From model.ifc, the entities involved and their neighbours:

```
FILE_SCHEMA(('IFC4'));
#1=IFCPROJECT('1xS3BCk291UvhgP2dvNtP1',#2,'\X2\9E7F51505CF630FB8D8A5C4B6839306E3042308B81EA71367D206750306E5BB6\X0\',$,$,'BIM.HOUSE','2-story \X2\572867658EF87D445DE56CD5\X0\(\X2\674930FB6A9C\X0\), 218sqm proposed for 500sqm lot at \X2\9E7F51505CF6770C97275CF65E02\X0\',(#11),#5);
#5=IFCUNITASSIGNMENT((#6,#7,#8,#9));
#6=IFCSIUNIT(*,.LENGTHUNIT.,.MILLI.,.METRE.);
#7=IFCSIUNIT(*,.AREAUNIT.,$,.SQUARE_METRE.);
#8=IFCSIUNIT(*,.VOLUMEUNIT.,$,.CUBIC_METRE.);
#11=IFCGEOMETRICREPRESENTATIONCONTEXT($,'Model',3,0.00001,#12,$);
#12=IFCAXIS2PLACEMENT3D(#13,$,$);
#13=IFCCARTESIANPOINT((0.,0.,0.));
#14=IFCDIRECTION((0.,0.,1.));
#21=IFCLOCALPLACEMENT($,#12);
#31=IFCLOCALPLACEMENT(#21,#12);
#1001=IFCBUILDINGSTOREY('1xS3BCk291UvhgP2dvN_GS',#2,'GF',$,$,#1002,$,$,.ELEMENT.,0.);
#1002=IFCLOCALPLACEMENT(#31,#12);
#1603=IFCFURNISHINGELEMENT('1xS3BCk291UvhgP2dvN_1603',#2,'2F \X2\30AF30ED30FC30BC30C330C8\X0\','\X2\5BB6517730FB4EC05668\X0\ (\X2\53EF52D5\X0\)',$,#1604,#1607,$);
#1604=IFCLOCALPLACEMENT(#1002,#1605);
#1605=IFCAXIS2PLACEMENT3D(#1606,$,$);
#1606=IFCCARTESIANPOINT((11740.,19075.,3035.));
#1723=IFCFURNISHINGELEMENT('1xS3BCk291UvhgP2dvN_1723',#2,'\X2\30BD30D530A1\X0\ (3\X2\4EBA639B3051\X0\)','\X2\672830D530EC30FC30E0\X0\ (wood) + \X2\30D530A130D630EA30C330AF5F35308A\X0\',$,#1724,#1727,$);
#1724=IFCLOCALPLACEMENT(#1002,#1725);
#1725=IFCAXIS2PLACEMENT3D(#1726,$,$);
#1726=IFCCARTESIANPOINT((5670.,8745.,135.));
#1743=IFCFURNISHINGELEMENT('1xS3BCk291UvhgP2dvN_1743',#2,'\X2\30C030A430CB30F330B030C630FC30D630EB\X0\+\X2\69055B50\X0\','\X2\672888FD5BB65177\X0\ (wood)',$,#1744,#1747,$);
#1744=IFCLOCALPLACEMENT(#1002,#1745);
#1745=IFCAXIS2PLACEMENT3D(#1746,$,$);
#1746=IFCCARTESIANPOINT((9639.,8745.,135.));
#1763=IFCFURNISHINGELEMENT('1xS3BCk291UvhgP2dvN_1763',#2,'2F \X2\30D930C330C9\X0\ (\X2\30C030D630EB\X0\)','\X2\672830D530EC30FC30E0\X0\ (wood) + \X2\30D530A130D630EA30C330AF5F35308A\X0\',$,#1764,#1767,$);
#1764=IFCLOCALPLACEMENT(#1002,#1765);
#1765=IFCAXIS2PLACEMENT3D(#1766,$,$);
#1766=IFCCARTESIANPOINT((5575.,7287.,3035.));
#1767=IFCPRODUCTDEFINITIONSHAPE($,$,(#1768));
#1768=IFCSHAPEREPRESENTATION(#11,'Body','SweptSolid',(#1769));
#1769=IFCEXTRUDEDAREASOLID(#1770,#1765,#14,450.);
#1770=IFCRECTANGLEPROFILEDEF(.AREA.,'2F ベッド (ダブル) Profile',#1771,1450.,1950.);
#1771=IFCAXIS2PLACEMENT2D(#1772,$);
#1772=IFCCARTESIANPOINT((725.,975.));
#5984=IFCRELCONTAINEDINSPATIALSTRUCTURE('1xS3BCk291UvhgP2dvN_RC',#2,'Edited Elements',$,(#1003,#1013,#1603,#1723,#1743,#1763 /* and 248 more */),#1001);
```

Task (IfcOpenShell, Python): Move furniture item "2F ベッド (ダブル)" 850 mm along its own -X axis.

```python
import ifcopenshell
import ifcopenshell.api.geometry
import ifcopenshell.util.placement
import ifcopenshell.util.unit

model = ifcopenshell.open("model.ifc")
unit_scale = ifcopenshell.util.unit.calculate_unit_scale(model)

item = model.by_guid("1xS3BCk291UvhgP2dvN_1763")
matrix = ifcopenshell.util.placement.get_local_placement(item.ObjectPlacement)
matrix[:3, 3] -= matrix[:3, 0] * 0.85 / unit_scale
ifcopenshell.api.geometry.edit_object_placement(model, product=item, matrix=matrix, is_si=False)

print(ifcopenshell.util.placement.get_local_placement(item.ObjectPlacement).round(3) + 0.0)

model.write("model_v2.ifc")
```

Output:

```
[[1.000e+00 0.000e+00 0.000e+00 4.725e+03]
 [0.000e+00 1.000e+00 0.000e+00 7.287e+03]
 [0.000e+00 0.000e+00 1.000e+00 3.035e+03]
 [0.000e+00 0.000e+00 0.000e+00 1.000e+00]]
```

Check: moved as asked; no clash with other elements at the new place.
